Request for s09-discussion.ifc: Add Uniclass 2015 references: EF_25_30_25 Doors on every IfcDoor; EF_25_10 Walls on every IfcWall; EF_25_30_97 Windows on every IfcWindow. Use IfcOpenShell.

First a look at what the model holds.

```python
import ifcopenshell

model = ifcopenshell.open("s09-discussion.ifc")
print(model.schema)
print("classifications:", [c.Name for c in model.by_type("IfcClassification")])
for ifc_class in ("IfcDoor", "IfcRoof", "IfcStair", "IfcWall", "IfcWindow"):
    print(ifc_class, len(model.by_type(ifc_class)))
```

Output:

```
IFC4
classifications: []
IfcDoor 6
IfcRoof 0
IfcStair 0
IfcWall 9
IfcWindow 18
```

```python
import ifcopenshell
import ifcopenshell.api.classification

model = ifcopenshell.open("s09-discussion.ifc")

system = ifcopenshell.api.classification.add_classification(model, classification="Uniclass 2015")

codes = {
    "IfcDoor": ("EF_25_30_25", "Doors"),
    "IfcWall": ("EF_25_10", "Walls"),
    "IfcWindow": ("EF_25_30_97", "Windows"),
}
for ifc_class, (code, name) in codes.items():
    products = model.by_type(ifc_class)
    ifcopenshell.api.classification.add_reference(
        model, products=products, classification=system, identification=code, name=name
    )
    print(code, len(products))

model.write("s09-discussion_updated.ifc")
```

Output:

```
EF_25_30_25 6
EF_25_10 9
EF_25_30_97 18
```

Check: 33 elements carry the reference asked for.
